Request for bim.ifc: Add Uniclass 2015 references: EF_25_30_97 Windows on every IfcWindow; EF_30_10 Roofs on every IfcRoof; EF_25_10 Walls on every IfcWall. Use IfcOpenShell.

First a look at what the model holds.

```python
import ifcopenshell

model = ifcopenshell.open("bim.ifc")
print(model.schema)
print("classifications:", [c.Name for c in model.by_type("IfcClassification")])
for ifc_class in ("IfcDoor", "IfcRoof", "IfcStair", "IfcWall", "IfcWindow"):
    print(ifc_class, len(model.by_type(ifc_class)))
```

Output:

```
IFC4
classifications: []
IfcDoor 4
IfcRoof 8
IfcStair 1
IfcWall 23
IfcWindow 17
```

```python
import ifcopenshell
import ifcopenshell.api.classification

model = ifcopenshell.open("bim.ifc")

system = ifcopenshell.api.classification.add_classification(model, classification="Uniclass 2015")

codes = {
    "IfcWindow": ("EF_25_30_97", "Windows"),
    "IfcRoof": ("EF_30_10", "Roofs"),
    "IfcWall": ("EF_25_10", "Walls"),
}
for ifc_class, (code, name) in codes.items():
    products = model.by_type(ifc_class)
    ifcopenshell.api.classification.add_reference(
        model, products=products, classification=system, identification=code, name=name
    )
    print(code, len(products))

model.write("bim_edited.ifc")
```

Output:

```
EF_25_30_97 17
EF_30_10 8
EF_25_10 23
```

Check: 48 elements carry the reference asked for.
